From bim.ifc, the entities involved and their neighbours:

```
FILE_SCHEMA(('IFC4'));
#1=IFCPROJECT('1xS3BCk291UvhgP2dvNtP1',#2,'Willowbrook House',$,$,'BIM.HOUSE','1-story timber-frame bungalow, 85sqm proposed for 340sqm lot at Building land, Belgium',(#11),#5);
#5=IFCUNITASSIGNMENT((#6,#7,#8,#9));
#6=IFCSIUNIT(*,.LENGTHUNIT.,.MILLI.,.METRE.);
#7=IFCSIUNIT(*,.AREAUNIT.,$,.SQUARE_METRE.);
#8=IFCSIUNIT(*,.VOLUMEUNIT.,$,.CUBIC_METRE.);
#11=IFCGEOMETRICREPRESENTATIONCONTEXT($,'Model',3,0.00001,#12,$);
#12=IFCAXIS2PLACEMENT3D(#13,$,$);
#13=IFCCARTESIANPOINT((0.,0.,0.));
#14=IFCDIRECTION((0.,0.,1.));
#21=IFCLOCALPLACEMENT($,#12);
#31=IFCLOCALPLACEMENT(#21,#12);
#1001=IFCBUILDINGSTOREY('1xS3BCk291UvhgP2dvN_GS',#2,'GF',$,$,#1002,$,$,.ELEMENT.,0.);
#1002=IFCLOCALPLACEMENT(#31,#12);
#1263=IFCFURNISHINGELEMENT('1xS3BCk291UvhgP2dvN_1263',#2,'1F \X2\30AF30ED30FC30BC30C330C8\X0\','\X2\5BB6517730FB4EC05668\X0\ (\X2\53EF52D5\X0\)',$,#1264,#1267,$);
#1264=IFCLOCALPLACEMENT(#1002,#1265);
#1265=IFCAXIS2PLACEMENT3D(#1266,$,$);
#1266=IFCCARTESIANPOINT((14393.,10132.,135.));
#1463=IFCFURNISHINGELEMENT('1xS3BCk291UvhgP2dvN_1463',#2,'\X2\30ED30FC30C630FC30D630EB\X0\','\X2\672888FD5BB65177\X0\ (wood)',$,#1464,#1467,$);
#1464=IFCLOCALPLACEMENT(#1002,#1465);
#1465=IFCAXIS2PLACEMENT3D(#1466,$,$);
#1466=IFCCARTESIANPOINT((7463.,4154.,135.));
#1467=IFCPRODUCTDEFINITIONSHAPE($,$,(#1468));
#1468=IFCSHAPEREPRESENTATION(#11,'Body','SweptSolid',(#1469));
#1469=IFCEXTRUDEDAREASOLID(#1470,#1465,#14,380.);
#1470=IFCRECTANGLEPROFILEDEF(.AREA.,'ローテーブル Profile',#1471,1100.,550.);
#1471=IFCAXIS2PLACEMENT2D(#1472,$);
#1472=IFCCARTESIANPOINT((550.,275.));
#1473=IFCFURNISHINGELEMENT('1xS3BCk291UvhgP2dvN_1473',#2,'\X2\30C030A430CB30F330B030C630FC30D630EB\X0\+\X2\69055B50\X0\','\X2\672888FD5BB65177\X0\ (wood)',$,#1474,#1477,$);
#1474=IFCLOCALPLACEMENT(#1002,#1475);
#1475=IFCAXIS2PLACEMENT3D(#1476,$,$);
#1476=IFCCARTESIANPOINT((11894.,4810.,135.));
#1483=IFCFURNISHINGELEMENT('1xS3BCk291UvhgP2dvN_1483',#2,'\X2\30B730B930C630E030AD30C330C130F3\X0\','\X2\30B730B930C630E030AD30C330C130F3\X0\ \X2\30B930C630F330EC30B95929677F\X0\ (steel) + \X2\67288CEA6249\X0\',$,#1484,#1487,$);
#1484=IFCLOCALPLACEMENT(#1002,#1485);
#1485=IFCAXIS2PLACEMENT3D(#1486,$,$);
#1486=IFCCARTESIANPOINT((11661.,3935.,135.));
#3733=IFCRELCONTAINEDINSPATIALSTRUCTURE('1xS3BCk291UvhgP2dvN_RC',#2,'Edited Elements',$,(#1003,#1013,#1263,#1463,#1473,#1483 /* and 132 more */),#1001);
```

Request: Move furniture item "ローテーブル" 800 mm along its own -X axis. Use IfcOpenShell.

```python
import ifcopenshell
import ifcopenshell.api.geometry
import ifcopenshell.util.placement

model = ifcopenshell.open("bim.ifc")

item = model.by_guid("1xS3BCk291UvhgP2dvN_1463")
matrix = ifcopenshell.util.placement.get_local_placement(item.ObjectPlacement)
matrix[:3, 3] -= matrix[:3, 0] * 800.0
ifcopenshell.api.geometry.edit_object_placement(model, product=item, matrix=matrix, is_si=False)

print(ifcopenshell.util.placement.get_local_placement(item.ObjectPlacement).round(3) + 0.0)

model.write("bim_edited.ifc")
```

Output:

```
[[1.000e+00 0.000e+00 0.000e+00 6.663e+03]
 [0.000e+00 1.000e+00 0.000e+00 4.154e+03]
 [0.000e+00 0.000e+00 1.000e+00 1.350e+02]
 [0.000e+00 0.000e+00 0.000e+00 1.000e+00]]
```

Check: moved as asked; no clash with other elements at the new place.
